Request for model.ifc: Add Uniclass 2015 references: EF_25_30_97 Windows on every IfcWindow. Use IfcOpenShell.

First a look at what the model holds.

```python
import ifcopenshell

model = ifcopenshell.open("model.ifc")
print(model.schema)
print("classifications:", [c.Name for c in model.by_type("IfcClassification")])
for ifc_class in ("IfcDoor", "IfcRoof", "IfcStair", "IfcWall", "IfcWindow"):
    print(ifc_class, len(model.by_type(ifc_class)))
```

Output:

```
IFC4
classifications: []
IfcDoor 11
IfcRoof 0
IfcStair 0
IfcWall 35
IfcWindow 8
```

```python
import ifcopenshell
import ifcopenshell.api.classification

model = ifcopenshell.open("model.ifc")

system = ifcopenshell.api.classification.add_classification(model, classification="Uniclass 2015")

codes = {
    "IfcWindow": ("EF_25_30_97", "Windows"),
}
for ifc_class, (code, name) in codes.items():
    products = model.by_type(ifc_class)
    ifcopenshell.api.classification.add_reference(
        model, products=products, classification=system, identification=code, name=name
    )
    print(code, len(products))

model.write("model-out.ifc")
```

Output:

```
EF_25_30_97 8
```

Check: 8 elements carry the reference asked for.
